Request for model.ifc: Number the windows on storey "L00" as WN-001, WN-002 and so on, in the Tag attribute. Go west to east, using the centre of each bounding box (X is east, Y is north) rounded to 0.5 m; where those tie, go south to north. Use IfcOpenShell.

First a look at what the model holds.

```python
import ifcopenshell
import ifcopenshell.util.element
import ifcopenshell.util.placement

model = ifcopenshell.open("model.ifc")
print(model.schema)
storey = next(s for s in model.by_type("IfcBuildingStorey") if s.Name == "L00")
windows = [e for e in ifcopenshell.util.element.get_decomposition(storey) if e.is_a("IfcWindow")]
for e in sorted(windows, key=lambda e: e.id()):
    origin = ifcopenshell.util.placement.get_local_placement(e.ObjectPlacement)[:3, 3]
    print(e.id(), e.Tag, e.Name, origin.round(2) + 0.0, sep=" | ")
```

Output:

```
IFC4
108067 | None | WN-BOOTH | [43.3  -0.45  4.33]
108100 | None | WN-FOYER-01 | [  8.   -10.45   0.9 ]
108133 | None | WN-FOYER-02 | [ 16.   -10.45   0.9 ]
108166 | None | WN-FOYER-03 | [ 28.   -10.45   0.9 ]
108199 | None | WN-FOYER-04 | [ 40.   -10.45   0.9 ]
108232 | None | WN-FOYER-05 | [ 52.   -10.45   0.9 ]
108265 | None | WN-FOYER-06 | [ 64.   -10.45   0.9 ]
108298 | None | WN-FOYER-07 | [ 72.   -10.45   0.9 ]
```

```python
import ifcopenshell
import ifcopenshell.geom
import ifcopenshell.util.element
import ifcopenshell.util.shape

model = ifcopenshell.open("model.ifc")
settings = ifcopenshell.geom.settings()
settings.set("use-world-coords", True)


def centre(element):
    shape = ifcopenshell.geom.create_shape(settings, element)
    return ifcopenshell.util.shape.get_bbox_centroid(shape.geometry)


storey = next(s for s in model.by_type("IfcBuildingStorey") if s.Name == "L00")
windows = [e for e in ifcopenshell.util.element.get_decomposition(storey) if e.is_a("IfcWindow")]

# Insertion points can sit at a corner or the storey origin, so sort by the geometry (in metres).
centres = {e: centre(e) for e in windows}
windows.sort(key=lambda e: (round(centres[e][0] / 0.5), centres[e][1]))

for i, e in enumerate(windows, start=1):
    number = f"WN-0{i:02d}"
    e.Tag = number
    print(e.id(), number)

model.write("model_updated.ifc")
```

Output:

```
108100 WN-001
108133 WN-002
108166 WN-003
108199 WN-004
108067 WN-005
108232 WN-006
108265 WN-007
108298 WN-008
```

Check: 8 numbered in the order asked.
